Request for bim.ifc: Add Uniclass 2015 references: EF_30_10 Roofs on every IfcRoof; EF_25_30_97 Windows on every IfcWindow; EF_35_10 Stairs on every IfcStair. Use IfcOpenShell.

First a look at what the model holds.

```python
import ifcopenshell

model = ifcopenshell.open("bim.ifc")
print(model.schema)
print("classifications:", [c.Name for c in model.by_type("IfcClassification")])
for ifc_class in ("IfcDoor", "IfcRoof", "IfcStair", "IfcWall", "IfcWindow"):
    print(ifc_class, len(model.by_type(ifc_class)))
```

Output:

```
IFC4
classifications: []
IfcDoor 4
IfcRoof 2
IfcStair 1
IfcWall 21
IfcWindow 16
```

```python
import ifcopenshell
import ifcopenshell.api.classification

model = ifcopenshell.open("bim.ifc")

system = ifcopenshell.api.classification.add_classification(model, classification="Uniclass 2015")

codes = {
    "IfcRoof": ("EF_30_10", "Roofs"),
    "IfcWindow": ("EF_25_30_97", "Windows"),
    "IfcStair": ("EF_35_10", "Stairs"),
}
for ifc_class, (code, name) in codes.items():
    products = model.by_type(ifc_class)
    ifcopenshell.api.classification.add_reference(
        model, products=products, classification=system, identification=code, name=name
    )
    print(code, len(products))

model.write("bim_edited.ifc")
```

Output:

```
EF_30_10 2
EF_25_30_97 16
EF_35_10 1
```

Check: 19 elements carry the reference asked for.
